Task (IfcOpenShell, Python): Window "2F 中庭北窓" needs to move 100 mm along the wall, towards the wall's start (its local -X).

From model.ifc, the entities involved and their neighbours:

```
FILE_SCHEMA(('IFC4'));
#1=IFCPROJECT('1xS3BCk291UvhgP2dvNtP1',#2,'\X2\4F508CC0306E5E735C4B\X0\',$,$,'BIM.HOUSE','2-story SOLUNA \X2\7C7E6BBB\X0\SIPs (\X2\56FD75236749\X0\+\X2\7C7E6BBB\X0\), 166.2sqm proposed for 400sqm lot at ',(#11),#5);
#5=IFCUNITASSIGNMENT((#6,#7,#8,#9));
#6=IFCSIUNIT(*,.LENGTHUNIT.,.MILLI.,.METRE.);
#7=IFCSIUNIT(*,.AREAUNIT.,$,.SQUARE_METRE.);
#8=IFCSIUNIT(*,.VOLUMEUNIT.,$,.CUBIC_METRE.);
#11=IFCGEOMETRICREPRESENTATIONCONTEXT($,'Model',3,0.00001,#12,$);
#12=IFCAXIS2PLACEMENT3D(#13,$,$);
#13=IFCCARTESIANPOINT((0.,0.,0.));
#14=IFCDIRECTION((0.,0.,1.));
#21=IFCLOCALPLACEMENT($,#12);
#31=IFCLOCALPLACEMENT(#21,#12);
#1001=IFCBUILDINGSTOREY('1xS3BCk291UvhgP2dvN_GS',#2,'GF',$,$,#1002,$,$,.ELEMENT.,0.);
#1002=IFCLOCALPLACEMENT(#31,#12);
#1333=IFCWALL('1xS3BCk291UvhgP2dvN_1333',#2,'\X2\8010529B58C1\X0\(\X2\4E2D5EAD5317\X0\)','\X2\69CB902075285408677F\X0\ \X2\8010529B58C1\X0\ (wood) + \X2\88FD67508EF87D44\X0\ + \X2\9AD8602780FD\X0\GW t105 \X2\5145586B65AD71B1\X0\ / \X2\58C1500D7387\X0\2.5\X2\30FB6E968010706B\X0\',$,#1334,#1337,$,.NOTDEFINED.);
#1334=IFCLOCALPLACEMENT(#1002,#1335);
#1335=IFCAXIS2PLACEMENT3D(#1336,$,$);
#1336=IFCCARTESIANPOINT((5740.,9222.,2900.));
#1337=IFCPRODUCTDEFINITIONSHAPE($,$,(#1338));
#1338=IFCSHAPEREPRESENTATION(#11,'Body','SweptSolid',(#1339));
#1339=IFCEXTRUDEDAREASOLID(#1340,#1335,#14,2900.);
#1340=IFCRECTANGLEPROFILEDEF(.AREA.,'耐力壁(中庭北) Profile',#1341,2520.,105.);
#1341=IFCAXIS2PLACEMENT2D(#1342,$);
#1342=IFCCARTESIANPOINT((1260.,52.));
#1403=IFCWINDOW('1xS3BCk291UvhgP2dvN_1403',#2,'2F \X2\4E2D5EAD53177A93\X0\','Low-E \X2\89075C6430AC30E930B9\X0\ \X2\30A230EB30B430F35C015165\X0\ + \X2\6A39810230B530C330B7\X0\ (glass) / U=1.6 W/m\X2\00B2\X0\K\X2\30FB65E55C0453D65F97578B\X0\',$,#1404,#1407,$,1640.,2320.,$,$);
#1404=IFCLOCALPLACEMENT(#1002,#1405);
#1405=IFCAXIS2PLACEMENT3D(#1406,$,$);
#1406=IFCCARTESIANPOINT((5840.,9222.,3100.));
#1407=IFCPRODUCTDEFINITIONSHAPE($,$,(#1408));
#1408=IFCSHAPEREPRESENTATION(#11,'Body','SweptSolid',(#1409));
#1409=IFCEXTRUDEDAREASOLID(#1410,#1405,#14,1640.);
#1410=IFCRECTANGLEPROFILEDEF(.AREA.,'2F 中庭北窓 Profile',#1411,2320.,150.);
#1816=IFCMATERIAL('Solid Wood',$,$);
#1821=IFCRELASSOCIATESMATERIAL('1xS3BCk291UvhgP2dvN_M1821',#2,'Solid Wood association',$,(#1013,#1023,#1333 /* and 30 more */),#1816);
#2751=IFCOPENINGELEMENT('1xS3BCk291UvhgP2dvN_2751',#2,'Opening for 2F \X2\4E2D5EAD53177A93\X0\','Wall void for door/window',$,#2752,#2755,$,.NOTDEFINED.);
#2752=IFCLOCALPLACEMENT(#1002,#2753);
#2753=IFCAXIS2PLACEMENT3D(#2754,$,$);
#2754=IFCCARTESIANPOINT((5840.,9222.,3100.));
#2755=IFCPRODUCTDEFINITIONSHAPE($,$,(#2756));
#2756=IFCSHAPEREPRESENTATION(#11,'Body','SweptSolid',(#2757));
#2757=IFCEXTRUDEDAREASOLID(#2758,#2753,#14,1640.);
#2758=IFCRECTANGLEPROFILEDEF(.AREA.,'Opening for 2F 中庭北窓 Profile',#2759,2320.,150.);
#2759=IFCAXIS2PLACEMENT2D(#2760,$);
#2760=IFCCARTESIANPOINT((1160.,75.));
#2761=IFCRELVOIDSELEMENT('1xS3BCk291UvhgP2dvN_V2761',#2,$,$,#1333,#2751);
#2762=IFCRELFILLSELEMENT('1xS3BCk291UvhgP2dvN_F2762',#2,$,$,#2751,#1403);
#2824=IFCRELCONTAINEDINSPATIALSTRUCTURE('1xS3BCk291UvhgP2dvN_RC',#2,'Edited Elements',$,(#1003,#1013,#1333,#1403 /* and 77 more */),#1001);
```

```python
import ifcopenshell
import ifcopenshell.api.geometry
import ifcopenshell.util.placement
import ifcopenshell.util.unit

model = ifcopenshell.open("model.ifc")
unit_scale = ifcopenshell.util.unit.calculate_unit_scale(model)

window = model.by_guid("1xS3BCk291UvhgP2dvN_1403")
opening = window.FillsVoids[0].RelatingOpeningElement
wall = opening.VoidsElements[0].RelatingBuildingElement

wall_matrix = ifcopenshell.util.placement.get_local_placement(wall.ObjectPlacement)
shift = wall_matrix[:3, 0] * -0.1 / unit_scale
before = ifcopenshell.util.placement.get_local_placement(window.ObjectPlacement)[:3, 3].copy()

# The window is not placed relative to its opening, so move both.
for product in (opening, window):
    matrix = ifcopenshell.util.placement.get_local_placement(product.ObjectPlacement)
    matrix[:3, 3] += shift
    ifcopenshell.api.geometry.edit_object_placement(model, product=product, matrix=matrix, is_si=False)

after = ifcopenshell.util.placement.get_local_placement(window.ObjectPlacement)[:3, 3]
print("window moved by", (after - before).round(3) + 0.0)

model.write("model_updated.ifc")
```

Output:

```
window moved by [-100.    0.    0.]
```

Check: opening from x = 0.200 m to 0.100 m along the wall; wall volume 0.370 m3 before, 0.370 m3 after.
